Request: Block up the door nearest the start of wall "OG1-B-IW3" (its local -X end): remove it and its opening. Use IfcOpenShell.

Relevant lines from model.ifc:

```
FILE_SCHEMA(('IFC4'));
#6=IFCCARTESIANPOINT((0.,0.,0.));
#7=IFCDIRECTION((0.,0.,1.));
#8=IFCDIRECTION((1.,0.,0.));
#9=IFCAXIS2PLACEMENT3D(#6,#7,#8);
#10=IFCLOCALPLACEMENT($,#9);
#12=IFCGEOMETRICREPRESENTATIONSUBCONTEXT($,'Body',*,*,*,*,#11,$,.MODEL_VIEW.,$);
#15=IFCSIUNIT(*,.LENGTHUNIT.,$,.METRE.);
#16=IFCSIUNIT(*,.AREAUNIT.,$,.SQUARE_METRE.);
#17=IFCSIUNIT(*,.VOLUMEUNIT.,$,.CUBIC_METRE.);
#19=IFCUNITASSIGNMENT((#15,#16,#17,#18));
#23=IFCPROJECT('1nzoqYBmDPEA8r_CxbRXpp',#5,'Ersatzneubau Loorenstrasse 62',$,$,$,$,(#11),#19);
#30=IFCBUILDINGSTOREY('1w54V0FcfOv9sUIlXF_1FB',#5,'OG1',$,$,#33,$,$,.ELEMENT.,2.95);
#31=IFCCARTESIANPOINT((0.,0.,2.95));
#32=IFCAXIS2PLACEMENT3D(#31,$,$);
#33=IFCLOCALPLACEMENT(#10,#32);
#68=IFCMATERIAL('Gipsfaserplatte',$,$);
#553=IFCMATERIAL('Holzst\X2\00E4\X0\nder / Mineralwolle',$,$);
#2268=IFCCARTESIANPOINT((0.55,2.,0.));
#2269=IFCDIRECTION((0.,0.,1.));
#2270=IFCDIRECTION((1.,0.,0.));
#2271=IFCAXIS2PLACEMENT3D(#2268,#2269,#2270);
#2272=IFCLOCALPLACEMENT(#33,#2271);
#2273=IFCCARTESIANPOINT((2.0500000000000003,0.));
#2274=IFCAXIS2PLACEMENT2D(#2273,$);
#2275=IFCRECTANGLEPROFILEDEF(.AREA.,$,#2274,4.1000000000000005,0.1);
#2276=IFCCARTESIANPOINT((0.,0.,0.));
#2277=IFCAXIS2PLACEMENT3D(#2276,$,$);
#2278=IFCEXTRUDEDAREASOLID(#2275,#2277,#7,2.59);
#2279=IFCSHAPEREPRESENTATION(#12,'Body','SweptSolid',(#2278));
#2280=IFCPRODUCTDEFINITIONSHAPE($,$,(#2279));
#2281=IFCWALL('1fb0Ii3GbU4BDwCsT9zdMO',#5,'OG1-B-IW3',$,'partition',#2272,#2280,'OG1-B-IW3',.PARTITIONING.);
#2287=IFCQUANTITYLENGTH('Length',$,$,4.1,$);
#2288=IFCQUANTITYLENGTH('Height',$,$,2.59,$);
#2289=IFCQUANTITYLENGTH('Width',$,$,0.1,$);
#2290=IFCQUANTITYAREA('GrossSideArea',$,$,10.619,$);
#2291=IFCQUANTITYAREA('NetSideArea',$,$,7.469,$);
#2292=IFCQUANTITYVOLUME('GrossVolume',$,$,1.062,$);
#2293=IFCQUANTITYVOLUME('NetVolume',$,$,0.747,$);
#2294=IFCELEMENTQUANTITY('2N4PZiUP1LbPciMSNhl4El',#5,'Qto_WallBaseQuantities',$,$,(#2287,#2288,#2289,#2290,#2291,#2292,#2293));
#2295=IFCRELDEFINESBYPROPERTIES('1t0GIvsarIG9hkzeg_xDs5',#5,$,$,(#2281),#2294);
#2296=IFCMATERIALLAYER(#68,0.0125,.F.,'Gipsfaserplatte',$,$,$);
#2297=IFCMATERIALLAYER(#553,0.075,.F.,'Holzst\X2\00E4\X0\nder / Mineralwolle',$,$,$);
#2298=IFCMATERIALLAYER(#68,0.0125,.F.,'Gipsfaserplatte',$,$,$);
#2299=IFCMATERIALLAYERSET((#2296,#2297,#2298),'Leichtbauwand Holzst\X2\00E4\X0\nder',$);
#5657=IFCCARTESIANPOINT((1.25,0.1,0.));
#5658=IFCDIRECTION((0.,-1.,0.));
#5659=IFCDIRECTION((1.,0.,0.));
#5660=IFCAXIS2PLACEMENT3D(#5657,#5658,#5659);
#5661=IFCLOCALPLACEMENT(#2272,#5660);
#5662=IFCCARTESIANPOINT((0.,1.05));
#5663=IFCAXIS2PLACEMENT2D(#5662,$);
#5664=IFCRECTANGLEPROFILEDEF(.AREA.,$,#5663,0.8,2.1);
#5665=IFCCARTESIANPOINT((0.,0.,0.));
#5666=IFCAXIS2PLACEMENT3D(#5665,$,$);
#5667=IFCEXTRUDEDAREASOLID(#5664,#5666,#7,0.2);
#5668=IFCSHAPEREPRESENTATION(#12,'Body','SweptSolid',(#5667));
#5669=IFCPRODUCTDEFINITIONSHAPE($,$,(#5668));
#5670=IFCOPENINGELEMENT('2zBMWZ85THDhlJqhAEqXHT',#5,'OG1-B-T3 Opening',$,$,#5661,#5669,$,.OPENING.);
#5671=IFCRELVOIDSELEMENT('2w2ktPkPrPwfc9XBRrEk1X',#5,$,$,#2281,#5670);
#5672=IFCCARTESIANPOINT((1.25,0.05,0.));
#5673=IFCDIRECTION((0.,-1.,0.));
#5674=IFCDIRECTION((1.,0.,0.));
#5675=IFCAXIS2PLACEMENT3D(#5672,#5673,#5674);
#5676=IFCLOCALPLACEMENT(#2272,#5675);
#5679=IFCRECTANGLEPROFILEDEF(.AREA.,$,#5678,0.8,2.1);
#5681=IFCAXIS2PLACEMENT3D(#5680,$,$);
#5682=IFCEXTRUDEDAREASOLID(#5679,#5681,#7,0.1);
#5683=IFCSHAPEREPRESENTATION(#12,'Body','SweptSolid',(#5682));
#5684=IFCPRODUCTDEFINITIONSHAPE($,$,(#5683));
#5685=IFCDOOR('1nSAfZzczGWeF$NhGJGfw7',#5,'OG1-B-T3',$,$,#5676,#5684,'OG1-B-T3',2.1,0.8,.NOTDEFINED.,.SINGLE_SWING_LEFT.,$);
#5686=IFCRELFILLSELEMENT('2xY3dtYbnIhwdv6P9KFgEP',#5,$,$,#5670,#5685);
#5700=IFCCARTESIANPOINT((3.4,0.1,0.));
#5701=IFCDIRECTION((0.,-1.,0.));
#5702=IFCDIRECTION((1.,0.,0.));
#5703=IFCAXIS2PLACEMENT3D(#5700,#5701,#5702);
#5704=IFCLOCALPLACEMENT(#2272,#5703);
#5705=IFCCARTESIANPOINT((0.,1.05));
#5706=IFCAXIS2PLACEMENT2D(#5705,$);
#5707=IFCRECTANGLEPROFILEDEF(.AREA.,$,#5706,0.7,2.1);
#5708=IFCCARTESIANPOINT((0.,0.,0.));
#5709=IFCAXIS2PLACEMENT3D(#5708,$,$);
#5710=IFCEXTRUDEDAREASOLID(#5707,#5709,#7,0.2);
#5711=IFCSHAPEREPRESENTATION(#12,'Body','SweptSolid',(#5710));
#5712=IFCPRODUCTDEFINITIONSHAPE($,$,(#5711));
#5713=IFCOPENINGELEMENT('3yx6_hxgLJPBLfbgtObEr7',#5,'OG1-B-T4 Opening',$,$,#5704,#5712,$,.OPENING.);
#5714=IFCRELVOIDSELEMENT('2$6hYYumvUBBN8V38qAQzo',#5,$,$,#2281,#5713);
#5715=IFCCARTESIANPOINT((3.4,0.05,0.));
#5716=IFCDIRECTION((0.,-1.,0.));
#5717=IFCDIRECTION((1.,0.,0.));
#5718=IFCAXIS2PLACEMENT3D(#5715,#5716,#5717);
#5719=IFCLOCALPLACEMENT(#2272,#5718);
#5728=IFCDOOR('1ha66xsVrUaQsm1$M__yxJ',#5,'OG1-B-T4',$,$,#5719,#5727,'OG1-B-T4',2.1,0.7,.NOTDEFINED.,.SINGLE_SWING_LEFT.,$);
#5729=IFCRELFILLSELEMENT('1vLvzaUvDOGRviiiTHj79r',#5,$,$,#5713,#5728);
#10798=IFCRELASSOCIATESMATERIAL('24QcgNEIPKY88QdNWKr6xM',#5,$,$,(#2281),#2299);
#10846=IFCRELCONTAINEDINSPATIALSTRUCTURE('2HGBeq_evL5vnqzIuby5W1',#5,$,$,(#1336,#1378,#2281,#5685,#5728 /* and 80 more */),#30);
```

```python
import ifcopenshell
import ifcopenshell.api.feature
import ifcopenshell.api.pset
import ifcopenshell.api.root
import ifcopenshell.geom
import ifcopenshell.util.element
import ifcopenshell.util.shape
import ifcopenshell.util.unit

model = ifcopenshell.open("model.ifc")
area_scale = ifcopenshell.util.unit.calculate_unit_scale(model, "AREAUNIT")
volume_scale = ifcopenshell.util.unit.calculate_unit_scale(model, "VOLUMEUNIT")
settings = ifcopenshell.geom.settings()


def volume(element):
    """Net volume in cubic metres, openings subtracted."""
    shape = ifcopenshell.geom.create_shape(settings, element)
    return ifcopenshell.util.shape.get_volume(shape.geometry)


door = model.by_guid("1nSAfZzczGWeF$NhGJGfw7")
opening = door.FillsVoids[0].RelatingOpeningElement
wall = opening.VoidsElements[0].RelatingBuildingElement
before = volume(wall)

ifcopenshell.api.root.remove_product(model, product=door)
ifcopenshell.api.feature.remove_feature(model, feature=opening)

after = volume(wall)
thickness = 0.1  # wall thickness in metres

# Update the wall's stored quantities.
qto = model.by_id(ifcopenshell.util.element.get_pset(wall, "Qto_WallBaseQuantities", should_inherit=False)["id"])
ifcopenshell.api.pset.edit_qto(model, qto=qto, properties={
    "NetSideArea": after / thickness / area_scale,
    "NetVolume": after / volume_scale,
})

print(f"wall volume {before:.3f} -> {after:.3f} m3")

model.write("model_v2.ifc")
```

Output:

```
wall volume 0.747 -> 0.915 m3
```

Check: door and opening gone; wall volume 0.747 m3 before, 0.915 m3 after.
